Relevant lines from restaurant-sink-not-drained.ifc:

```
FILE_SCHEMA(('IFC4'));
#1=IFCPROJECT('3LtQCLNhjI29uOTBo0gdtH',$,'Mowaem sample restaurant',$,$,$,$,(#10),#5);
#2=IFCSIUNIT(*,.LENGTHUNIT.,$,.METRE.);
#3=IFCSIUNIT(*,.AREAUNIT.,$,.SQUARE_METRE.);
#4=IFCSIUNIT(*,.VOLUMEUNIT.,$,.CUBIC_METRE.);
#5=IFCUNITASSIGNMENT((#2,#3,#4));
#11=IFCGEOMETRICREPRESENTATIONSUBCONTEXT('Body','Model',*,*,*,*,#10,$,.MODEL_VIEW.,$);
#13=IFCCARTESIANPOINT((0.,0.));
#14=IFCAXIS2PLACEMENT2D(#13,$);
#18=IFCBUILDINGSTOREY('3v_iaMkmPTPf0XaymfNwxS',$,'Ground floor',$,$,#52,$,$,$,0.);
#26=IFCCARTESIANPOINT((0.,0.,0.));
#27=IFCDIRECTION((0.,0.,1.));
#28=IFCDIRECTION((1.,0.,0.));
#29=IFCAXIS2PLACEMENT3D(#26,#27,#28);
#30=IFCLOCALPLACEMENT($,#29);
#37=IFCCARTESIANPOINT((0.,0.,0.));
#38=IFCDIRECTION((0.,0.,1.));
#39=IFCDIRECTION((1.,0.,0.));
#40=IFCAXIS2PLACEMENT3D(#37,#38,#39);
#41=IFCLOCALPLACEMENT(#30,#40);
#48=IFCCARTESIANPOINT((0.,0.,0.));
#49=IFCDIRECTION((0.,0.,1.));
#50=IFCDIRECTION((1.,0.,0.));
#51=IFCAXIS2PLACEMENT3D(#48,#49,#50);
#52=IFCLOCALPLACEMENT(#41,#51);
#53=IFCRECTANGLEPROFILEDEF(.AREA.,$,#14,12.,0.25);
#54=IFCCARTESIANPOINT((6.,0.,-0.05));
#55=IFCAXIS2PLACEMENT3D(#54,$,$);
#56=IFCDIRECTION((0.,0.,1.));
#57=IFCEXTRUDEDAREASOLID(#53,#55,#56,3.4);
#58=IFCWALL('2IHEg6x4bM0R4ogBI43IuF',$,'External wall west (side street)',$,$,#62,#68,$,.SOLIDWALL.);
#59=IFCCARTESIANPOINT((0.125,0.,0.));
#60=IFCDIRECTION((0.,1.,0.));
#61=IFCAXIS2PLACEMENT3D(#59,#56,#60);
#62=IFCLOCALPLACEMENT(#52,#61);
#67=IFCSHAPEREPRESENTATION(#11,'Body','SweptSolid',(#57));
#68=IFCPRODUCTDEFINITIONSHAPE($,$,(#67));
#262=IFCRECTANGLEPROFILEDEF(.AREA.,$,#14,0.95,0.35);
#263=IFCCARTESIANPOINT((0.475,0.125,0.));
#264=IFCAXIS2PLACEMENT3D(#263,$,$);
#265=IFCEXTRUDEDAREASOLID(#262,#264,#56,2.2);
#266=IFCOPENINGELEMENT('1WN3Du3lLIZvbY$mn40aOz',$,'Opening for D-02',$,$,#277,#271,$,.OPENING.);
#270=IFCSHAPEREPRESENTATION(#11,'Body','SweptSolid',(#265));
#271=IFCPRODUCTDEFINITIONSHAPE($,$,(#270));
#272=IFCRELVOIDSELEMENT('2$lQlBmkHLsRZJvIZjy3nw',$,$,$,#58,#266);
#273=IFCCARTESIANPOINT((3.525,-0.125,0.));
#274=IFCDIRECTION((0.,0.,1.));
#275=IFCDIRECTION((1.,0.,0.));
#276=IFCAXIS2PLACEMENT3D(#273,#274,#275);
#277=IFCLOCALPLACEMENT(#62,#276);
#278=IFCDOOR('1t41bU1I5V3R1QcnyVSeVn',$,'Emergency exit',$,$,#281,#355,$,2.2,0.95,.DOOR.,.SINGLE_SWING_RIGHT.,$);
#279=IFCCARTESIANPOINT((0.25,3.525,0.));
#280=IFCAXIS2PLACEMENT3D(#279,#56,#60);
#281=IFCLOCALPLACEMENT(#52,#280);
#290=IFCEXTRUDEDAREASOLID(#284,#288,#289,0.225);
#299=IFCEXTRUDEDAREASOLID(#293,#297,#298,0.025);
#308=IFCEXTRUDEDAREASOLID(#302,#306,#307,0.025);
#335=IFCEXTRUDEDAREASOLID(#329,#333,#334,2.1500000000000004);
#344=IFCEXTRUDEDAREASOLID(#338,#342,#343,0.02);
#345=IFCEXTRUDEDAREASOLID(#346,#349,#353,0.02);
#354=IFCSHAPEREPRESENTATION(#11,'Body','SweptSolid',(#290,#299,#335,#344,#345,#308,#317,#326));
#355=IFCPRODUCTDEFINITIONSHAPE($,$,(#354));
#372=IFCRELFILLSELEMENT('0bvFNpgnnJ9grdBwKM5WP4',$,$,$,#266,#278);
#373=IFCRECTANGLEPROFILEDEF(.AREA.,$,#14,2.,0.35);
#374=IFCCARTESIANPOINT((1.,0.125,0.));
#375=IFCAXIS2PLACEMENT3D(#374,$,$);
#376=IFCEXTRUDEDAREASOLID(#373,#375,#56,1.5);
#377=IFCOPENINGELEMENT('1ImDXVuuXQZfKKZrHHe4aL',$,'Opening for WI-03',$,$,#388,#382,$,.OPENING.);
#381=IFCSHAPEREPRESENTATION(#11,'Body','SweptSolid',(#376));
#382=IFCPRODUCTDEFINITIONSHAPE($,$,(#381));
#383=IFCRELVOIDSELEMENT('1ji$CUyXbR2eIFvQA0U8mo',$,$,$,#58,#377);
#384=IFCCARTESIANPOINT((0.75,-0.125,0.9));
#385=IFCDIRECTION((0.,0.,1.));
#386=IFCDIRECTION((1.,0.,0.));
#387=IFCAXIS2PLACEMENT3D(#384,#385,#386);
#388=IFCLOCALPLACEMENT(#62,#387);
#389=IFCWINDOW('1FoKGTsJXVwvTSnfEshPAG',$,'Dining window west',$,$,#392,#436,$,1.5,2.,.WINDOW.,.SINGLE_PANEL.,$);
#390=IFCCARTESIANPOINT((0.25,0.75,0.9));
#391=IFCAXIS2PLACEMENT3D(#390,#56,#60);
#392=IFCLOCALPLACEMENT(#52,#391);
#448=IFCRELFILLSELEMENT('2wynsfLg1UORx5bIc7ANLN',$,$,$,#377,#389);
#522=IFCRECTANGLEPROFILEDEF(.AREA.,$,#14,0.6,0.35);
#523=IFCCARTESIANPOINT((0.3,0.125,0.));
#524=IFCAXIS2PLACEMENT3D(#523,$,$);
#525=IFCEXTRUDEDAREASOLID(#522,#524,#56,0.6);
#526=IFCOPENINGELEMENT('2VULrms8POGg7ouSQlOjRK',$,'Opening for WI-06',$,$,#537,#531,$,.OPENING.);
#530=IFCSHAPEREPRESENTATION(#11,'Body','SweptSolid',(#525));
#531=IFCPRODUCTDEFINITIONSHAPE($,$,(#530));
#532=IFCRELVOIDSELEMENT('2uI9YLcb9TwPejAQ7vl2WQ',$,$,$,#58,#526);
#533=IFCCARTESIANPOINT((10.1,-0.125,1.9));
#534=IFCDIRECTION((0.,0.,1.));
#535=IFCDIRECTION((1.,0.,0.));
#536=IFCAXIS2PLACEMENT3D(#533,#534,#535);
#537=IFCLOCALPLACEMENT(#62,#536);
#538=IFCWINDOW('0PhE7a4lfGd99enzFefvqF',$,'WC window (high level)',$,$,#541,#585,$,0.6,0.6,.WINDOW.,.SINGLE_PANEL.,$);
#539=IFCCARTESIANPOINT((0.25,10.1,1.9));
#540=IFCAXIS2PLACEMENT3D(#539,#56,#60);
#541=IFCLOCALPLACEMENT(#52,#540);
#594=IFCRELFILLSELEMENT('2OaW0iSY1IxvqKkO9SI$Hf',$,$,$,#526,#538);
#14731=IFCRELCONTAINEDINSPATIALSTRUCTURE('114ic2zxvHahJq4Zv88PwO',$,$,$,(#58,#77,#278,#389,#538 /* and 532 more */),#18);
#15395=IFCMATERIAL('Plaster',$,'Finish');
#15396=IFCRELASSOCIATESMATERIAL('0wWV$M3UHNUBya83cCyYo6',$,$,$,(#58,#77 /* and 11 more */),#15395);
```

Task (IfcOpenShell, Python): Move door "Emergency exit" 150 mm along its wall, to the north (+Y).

```python
import ifcopenshell
import ifcopenshell.api.geometry
import ifcopenshell.util.placement
import ifcopenshell.util.unit

model = ifcopenshell.open("restaurant-sink-not-drained.ifc")
unit_scale = ifcopenshell.util.unit.calculate_unit_scale(model)

door = model.by_id(278)
opening = door.FillsVoids[0].RelatingOpeningElement
wall = opening.VoidsElements[0].RelatingBuildingElement

wall_matrix = ifcopenshell.util.placement.get_local_placement(wall.ObjectPlacement)
shift = wall_matrix[:3, 0] * 0.15 / unit_scale
before = ifcopenshell.util.placement.get_local_placement(door.ObjectPlacement)[:3, 3].copy()

# The door is not placed relative to its opening, so move both.
for product in (opening, door):
    matrix = ifcopenshell.util.placement.get_local_placement(product.ObjectPlacement)
    matrix[:3, 3] += shift
    ifcopenshell.api.geometry.edit_object_placement(model, product=product, matrix=matrix, is_si=False)

after = ifcopenshell.util.placement.get_local_placement(door.ObjectPlacement)[:3, 3]
print("door moved by", (after - before).round(3) + 0.0)

model.write("restaurant-sink-not-drained_v2.ifc")
```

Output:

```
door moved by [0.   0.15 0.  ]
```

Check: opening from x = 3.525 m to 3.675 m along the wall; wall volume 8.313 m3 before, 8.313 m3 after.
